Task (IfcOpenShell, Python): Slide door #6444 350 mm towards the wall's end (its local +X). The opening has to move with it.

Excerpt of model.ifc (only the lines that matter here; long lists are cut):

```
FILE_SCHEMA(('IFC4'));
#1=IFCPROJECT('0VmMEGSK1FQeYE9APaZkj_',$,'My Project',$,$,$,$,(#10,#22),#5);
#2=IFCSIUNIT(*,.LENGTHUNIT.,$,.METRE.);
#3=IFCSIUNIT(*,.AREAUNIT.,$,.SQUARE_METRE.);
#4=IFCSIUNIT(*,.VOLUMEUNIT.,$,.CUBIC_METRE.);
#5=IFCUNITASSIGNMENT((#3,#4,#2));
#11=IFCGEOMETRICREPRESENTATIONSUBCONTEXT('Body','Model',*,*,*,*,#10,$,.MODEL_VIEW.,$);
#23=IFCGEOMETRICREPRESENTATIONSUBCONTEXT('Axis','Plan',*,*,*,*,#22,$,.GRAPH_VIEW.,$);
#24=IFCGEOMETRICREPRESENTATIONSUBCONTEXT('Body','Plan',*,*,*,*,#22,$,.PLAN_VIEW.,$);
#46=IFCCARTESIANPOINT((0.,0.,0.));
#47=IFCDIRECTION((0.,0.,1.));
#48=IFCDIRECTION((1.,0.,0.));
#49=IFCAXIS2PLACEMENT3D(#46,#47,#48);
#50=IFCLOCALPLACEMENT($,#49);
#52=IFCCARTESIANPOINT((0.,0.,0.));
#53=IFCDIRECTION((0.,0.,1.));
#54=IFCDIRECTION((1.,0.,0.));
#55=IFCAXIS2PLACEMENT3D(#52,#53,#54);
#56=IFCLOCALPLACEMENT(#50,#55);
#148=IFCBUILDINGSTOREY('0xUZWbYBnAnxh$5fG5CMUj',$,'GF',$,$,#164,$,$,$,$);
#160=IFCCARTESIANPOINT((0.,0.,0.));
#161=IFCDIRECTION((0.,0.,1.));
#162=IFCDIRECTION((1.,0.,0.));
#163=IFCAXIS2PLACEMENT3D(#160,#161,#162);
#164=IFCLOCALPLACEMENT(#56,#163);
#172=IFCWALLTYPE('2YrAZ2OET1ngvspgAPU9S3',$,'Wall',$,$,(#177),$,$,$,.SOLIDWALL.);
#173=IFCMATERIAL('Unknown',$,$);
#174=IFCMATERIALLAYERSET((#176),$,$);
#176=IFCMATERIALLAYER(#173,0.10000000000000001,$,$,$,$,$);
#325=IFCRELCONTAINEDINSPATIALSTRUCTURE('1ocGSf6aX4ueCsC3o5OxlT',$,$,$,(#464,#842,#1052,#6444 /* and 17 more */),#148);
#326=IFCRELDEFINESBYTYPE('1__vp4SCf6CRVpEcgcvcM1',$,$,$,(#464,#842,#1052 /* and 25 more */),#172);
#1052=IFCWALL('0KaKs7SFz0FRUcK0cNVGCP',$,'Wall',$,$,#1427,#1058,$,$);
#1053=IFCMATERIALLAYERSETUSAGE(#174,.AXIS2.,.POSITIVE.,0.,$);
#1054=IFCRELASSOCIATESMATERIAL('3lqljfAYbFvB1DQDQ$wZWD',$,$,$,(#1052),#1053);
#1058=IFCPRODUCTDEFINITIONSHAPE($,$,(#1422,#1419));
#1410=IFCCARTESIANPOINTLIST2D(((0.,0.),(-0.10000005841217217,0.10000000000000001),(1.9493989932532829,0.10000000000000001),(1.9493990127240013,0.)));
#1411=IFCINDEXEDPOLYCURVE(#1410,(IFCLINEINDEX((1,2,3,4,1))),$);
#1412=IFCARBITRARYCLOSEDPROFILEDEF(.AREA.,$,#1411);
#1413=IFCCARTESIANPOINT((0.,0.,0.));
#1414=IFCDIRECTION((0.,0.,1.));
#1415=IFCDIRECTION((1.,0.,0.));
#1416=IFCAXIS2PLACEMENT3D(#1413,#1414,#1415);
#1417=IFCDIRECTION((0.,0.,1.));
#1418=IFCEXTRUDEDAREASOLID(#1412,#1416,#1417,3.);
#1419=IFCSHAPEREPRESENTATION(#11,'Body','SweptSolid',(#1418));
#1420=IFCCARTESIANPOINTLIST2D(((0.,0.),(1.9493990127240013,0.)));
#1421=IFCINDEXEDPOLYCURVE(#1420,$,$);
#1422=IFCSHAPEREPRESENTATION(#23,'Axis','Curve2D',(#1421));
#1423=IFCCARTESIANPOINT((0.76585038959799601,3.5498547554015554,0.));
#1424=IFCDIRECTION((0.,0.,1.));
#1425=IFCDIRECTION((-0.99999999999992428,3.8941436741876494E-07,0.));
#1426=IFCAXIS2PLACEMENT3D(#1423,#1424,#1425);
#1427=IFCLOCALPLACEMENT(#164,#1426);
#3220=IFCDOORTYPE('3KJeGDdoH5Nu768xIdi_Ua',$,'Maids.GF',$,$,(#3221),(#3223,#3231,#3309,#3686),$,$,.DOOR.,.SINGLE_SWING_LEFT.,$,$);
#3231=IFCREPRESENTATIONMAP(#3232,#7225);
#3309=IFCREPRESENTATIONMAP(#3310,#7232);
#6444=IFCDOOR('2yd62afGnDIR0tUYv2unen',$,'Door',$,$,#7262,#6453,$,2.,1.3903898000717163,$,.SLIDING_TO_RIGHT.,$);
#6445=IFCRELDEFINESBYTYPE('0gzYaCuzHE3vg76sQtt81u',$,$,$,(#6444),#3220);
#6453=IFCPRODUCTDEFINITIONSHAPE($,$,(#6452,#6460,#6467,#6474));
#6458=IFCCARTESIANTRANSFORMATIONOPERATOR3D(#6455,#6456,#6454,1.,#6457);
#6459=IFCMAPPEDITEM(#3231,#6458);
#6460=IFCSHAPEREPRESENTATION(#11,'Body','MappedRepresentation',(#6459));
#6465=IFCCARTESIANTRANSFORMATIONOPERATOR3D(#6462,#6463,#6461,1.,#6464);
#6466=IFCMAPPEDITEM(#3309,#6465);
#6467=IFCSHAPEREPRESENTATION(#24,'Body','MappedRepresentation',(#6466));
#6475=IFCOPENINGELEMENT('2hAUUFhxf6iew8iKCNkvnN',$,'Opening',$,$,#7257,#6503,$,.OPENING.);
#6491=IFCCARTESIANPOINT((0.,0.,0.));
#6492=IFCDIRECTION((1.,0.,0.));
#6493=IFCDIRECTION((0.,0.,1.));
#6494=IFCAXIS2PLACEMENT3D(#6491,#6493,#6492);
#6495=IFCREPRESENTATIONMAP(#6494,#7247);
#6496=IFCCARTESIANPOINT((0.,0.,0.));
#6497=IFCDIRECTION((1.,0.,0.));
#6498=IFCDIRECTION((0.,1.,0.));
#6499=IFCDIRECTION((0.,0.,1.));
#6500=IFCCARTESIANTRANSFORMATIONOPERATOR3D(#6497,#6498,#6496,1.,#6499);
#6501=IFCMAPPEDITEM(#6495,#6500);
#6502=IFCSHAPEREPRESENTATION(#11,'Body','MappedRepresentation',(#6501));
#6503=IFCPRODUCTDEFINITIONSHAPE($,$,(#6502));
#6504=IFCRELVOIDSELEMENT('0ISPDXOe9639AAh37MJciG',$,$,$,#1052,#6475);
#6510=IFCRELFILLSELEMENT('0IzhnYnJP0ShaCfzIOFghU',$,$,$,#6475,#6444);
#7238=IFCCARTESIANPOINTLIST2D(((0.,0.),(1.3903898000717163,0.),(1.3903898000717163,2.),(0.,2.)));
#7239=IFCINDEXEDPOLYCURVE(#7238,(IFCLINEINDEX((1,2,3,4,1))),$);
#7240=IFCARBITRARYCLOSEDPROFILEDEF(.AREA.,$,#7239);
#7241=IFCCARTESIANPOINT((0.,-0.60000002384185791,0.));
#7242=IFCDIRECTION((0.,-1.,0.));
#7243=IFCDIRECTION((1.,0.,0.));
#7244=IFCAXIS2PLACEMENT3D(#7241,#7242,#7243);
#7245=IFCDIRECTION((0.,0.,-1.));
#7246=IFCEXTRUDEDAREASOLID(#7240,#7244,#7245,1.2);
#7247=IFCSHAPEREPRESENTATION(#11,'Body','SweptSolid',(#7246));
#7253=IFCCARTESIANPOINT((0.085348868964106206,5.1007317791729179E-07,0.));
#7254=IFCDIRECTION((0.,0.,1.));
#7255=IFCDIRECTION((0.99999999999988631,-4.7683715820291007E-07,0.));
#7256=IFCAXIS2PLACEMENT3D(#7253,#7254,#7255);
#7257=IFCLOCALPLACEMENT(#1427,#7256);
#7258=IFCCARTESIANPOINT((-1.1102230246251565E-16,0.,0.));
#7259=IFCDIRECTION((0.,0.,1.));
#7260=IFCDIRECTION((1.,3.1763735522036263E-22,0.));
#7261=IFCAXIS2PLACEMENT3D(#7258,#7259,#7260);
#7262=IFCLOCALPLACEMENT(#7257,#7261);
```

```python
import ifcopenshell
import ifcopenshell.api.geometry
import ifcopenshell.util.placement
import ifcopenshell.util.unit

model = ifcopenshell.open("model.ifc")
unit_scale = ifcopenshell.util.unit.calculate_unit_scale(model)

door = model.by_guid("2yd62afGnDIR0tUYv2unen")
opening = door.FillsVoids[0].RelatingOpeningElement
wall = opening.VoidsElements[0].RelatingBuildingElement

wall_matrix = ifcopenshell.util.placement.get_local_placement(wall.ObjectPlacement)
shift = wall_matrix[:3, 0] * 0.35 / unit_scale
before = ifcopenshell.util.placement.get_local_placement(door.ObjectPlacement)[:3, 3].copy()

# The door is placed relative to its opening, so it follows when the opening moves.
matrix = ifcopenshell.util.placement.get_local_placement(opening.ObjectPlacement)
matrix[:3, 3] += shift
ifcopenshell.api.geometry.edit_object_placement(
    model, product=opening, matrix=matrix, is_si=False, should_transform_children=True
)

after = ifcopenshell.util.placement.get_local_placement(door.ObjectPlacement)[:3, 3]
print("door moved by", (after - before).round(3) + 0.0)

model.write("model_updated.ifc")
```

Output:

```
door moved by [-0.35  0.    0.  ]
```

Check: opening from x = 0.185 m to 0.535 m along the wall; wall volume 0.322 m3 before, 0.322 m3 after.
